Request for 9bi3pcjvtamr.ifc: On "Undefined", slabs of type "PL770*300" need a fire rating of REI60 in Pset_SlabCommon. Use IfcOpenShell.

First a look at what the model holds.

```python
import ifcopenshell
import ifcopenshell.util.element

model = ifcopenshell.open("9bi3pcjvtamr.ifc")
print(model.schema)
storey = next(s for s in model.by_type("IfcBuildingStorey") if s.Name == "Undefined")
slabs = [e for e in ifcopenshell.util.element.get_decomposition(storey) if e.is_a("IfcSlab")]
seen = {}
for e in slabs:
    element_type = ifcopenshell.util.element.get_type(e)
    key = (element_type.Name if element_type != e and element_type else None, ifcopenshell.util.element.get_pset(e, "Pset_SlabCommon", "FireRating"))
    seen[key] = seen.get(key, 0) + 1
for (name, value), count in sorted(seen.items(), key=str):
    print(count, "x", name, "|", value)
```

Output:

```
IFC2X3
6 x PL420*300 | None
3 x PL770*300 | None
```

```python
import ifcopenshell
import ifcopenshell.api.pset
import ifcopenshell.util.element

model = ifcopenshell.open("9bi3pcjvtamr.ifc")

storey = next(s for s in model.by_type("IfcBuildingStorey") if s.Name == "Undefined")
slabs = [e for e in ifcopenshell.util.element.get_decomposition(storey) if e.is_a("IfcSlab")]

count = 0
for e in slabs:
    element_type = ifcopenshell.util.element.get_type(e)
    if element_type in (None, e) or element_type.Name != "PL770*300":
        continue
    found = ifcopenshell.util.element.get_pset(e, "Pset_SlabCommon", should_inherit=False)
    if found:
        pset = model.by_id(found["id"])
        if len(ifcopenshell.util.element.get_elements_by_pset(pset)) > 1:
            pset = ifcopenshell.api.pset.unshare_pset(model, products=[e], pset=pset)[0]
    else:
        pset = ifcopenshell.api.pset.add_pset(model, product=e, name="Pset_SlabCommon")
    ifcopenshell.api.pset.edit_pset(model, pset=pset, properties={"FireRating": "REI60"})
    count += 1

print(count, "slabs updated")

model.write("9bi3pcjvtamr_v2.ifc")
```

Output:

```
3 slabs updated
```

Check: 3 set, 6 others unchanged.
